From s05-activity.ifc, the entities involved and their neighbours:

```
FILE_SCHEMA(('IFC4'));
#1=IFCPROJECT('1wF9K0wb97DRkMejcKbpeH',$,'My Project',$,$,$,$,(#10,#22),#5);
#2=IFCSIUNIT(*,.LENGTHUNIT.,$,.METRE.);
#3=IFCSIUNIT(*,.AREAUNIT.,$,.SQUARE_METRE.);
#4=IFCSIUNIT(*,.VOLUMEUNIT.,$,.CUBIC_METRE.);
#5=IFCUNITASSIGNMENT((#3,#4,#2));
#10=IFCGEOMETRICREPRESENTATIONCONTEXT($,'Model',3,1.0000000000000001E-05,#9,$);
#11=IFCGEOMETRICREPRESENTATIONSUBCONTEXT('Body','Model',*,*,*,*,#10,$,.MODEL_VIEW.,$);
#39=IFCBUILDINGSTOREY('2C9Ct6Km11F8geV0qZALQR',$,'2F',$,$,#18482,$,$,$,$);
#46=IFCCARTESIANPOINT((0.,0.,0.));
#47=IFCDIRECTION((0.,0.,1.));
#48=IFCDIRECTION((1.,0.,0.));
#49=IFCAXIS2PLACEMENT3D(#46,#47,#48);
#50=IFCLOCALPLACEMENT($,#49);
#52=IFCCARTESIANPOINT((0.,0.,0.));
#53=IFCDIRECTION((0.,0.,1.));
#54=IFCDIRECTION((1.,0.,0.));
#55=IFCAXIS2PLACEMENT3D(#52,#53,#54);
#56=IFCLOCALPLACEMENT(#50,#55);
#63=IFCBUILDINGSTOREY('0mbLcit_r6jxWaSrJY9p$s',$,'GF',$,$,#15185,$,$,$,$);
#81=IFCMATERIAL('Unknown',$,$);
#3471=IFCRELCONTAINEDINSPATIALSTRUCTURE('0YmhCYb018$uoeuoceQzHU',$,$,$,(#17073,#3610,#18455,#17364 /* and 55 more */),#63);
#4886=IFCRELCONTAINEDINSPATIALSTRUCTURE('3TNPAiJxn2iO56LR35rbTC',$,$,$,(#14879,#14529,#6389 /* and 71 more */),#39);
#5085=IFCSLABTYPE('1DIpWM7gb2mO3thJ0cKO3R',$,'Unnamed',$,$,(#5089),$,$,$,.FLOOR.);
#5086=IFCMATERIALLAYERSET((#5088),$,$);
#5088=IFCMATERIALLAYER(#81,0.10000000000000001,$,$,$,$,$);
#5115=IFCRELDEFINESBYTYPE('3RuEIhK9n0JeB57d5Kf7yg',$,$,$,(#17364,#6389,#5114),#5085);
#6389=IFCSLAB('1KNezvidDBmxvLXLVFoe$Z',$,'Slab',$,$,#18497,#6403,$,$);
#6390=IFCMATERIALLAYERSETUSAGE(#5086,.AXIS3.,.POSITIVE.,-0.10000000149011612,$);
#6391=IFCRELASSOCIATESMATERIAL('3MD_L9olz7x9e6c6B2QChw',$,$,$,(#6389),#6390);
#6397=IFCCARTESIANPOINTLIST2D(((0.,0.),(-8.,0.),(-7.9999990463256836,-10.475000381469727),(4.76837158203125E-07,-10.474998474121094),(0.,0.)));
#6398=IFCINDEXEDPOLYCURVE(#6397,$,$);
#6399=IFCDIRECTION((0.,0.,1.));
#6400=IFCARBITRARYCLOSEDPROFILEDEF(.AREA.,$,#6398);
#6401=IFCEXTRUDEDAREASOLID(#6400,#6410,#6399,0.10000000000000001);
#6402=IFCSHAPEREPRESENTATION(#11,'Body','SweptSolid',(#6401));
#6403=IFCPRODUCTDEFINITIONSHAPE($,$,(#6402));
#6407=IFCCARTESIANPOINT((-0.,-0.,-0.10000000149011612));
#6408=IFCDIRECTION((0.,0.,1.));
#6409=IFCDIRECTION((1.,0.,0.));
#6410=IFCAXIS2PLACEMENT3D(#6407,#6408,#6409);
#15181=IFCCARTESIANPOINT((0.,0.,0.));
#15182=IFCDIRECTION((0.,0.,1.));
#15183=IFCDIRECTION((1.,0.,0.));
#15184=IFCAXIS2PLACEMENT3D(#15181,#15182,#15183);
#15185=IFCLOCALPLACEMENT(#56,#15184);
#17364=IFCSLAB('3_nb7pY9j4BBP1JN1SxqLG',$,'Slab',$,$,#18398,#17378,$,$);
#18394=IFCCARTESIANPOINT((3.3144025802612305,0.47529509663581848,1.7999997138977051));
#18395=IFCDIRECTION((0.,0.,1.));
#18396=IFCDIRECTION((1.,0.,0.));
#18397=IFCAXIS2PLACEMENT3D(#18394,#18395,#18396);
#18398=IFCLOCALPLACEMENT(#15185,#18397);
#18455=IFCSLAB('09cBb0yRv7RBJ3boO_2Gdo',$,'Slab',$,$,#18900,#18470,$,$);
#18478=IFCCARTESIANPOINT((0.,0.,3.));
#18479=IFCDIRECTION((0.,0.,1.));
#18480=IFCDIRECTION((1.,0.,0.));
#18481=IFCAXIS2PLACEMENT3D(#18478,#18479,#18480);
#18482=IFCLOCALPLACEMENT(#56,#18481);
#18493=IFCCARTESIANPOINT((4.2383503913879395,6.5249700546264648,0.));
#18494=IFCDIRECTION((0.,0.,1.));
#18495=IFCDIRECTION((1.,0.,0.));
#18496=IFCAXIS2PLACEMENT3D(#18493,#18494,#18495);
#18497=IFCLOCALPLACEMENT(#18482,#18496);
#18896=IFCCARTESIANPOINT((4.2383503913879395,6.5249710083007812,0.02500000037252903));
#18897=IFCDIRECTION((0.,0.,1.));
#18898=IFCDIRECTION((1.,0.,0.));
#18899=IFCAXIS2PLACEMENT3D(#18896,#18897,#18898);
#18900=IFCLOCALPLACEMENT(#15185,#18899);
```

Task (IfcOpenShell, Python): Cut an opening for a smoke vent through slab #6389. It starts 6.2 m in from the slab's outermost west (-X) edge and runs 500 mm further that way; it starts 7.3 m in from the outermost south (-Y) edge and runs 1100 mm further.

```python
import numpy as np
import ifcopenshell
import ifcopenshell.api.feature
import ifcopenshell.api.geometry
import ifcopenshell.api.root
import ifcopenshell.geom
import ifcopenshell.util.placement
import ifcopenshell.util.representation
import ifcopenshell.util.shape
import ifcopenshell.util.unit

model = ifcopenshell.open("s05-activity.ifc")
unit_scale = ifcopenshell.util.unit.calculate_unit_scale(model)
settings = ifcopenshell.geom.settings()


def volume(element):
    """Net volume in cubic metres, openings subtracted."""
    shape = ifcopenshell.geom.create_shape(settings, element)
    return ifcopenshell.util.shape.get_volume(shape.geometry)


slab = model.by_guid("1KNezvidDBmxvLXLVFoe$Z")
before = volume(slab)

# Extent in the slab's own axes, in metres. The edges named are its -X and -Y sides.
slab_shape = ifcopenshell.geom.create_shape(settings, slab)
vertices = ifcopenshell.util.shape.get_vertices(slab_shape.geometry)
x_min, y_min, bottom = vertices.min(axis=0)
top = vertices[:, 2].max()

opening = ifcopenshell.api.root.create_entity(model, ifc_class="IfcOpeningElement", name="Smoke vent opening", predefined_type="OPENING")
context = ifcopenshell.util.representation.get_context(model, "Model", "Body", "MODEL_VIEW")
width, depth = 0.5, 1.1
outline = [(0.0, 0.0), (width, 0.0), (width, depth), (0.0, depth), (0.0, 0.0)]
# Overshoot both faces by 50 mm so the cut is clean.
shape = ifcopenshell.api.geometry.add_slab_representation(
    model, context=context, depth=top - bottom + 0.1, polyline=outline
)
ifcopenshell.api.geometry.assign_representation(model, product=opening, representation=shape)

matrix = ifcopenshell.util.placement.get_local_placement(slab.ObjectPlacement)
matrix[:, 3] = matrix @ np.append(np.array([x_min + 6.2, y_min + 7.3, bottom - 0.05]) / unit_scale, 1.0)
ifcopenshell.api.geometry.edit_object_placement(model, product=opening, matrix=matrix, is_si=False)
ifcopenshell.api.feature.add_feature(model, feature=opening, element=slab)

after = volume(slab)

print(f"slab volume {before:.3f} -> {after:.3f} m3")

model.write("s05-activity_rev.ifc")
```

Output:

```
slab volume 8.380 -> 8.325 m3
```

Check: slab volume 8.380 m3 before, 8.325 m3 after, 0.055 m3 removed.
